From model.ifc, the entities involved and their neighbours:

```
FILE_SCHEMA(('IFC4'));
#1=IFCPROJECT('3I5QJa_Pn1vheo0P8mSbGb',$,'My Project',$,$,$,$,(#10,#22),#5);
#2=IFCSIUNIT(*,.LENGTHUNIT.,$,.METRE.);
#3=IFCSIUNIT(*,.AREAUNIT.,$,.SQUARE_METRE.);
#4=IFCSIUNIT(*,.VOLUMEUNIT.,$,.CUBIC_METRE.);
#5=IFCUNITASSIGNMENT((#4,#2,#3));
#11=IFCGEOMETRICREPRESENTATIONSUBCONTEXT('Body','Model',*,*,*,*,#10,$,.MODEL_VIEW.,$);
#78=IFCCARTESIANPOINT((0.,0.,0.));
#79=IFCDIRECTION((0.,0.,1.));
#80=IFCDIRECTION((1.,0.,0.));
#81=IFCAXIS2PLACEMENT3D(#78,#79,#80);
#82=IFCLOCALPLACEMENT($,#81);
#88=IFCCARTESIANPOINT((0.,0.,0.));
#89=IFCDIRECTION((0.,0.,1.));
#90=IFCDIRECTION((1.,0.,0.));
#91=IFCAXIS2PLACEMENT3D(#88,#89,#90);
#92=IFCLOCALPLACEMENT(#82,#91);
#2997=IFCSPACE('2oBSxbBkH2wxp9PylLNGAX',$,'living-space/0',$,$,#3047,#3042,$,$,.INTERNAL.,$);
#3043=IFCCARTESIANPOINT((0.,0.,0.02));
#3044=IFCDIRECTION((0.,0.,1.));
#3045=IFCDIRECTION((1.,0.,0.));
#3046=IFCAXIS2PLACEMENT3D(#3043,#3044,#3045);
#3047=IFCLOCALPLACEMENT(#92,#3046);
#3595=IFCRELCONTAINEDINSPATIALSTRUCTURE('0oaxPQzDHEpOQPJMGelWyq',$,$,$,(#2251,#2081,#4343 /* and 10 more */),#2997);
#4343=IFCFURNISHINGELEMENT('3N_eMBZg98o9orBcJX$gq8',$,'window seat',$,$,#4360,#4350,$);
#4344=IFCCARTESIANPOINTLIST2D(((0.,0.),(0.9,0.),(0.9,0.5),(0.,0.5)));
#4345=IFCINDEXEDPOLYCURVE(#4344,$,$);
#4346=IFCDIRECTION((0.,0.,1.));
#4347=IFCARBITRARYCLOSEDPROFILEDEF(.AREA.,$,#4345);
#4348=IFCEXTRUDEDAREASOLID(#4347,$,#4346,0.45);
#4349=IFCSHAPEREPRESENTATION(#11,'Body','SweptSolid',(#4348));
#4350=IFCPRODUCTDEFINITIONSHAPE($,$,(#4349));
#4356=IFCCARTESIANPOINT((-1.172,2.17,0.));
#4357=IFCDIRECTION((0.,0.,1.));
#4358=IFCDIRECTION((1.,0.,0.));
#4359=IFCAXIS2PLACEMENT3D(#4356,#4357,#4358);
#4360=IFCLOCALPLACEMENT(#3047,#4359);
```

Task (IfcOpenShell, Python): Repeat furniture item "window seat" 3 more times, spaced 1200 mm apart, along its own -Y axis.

```python
import ifcopenshell
import ifcopenshell.api.geometry
import ifcopenshell.api.root
import ifcopenshell.util.element
import ifcopenshell.util.placement
import ifcopenshell.util.unit

model = ifcopenshell.open("model.ifc")
unit_scale = ifcopenshell.util.unit.calculate_unit_scale(model)

source = model.by_guid("3N_eMBZg98o9orBcJX$gq8")
base = ifcopenshell.util.placement.get_local_placement(source.ObjectPlacement)
step = -base[:3, 1] * 1.2 / unit_scale

for i in range(1, 4):
    copy = ifcopenshell.api.root.copy_class(model, product=source)
    copy.Representation = ifcopenshell.util.element.copy_deep(
        model, source.Representation, exclude=["IfcGeometricRepresentationContext", "IfcRepresentationMap"]
    )
    matrix = base.copy()
    matrix[:3, 3] += i * step
    print("added at", matrix[:3, 3].round(3) + 0.0)
    ifcopenshell.api.geometry.edit_object_placement(model, product=copy, matrix=matrix, is_si=False)

model.write("model_edited.ifc")
```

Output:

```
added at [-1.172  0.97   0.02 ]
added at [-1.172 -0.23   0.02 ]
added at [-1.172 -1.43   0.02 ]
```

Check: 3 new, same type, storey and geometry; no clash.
